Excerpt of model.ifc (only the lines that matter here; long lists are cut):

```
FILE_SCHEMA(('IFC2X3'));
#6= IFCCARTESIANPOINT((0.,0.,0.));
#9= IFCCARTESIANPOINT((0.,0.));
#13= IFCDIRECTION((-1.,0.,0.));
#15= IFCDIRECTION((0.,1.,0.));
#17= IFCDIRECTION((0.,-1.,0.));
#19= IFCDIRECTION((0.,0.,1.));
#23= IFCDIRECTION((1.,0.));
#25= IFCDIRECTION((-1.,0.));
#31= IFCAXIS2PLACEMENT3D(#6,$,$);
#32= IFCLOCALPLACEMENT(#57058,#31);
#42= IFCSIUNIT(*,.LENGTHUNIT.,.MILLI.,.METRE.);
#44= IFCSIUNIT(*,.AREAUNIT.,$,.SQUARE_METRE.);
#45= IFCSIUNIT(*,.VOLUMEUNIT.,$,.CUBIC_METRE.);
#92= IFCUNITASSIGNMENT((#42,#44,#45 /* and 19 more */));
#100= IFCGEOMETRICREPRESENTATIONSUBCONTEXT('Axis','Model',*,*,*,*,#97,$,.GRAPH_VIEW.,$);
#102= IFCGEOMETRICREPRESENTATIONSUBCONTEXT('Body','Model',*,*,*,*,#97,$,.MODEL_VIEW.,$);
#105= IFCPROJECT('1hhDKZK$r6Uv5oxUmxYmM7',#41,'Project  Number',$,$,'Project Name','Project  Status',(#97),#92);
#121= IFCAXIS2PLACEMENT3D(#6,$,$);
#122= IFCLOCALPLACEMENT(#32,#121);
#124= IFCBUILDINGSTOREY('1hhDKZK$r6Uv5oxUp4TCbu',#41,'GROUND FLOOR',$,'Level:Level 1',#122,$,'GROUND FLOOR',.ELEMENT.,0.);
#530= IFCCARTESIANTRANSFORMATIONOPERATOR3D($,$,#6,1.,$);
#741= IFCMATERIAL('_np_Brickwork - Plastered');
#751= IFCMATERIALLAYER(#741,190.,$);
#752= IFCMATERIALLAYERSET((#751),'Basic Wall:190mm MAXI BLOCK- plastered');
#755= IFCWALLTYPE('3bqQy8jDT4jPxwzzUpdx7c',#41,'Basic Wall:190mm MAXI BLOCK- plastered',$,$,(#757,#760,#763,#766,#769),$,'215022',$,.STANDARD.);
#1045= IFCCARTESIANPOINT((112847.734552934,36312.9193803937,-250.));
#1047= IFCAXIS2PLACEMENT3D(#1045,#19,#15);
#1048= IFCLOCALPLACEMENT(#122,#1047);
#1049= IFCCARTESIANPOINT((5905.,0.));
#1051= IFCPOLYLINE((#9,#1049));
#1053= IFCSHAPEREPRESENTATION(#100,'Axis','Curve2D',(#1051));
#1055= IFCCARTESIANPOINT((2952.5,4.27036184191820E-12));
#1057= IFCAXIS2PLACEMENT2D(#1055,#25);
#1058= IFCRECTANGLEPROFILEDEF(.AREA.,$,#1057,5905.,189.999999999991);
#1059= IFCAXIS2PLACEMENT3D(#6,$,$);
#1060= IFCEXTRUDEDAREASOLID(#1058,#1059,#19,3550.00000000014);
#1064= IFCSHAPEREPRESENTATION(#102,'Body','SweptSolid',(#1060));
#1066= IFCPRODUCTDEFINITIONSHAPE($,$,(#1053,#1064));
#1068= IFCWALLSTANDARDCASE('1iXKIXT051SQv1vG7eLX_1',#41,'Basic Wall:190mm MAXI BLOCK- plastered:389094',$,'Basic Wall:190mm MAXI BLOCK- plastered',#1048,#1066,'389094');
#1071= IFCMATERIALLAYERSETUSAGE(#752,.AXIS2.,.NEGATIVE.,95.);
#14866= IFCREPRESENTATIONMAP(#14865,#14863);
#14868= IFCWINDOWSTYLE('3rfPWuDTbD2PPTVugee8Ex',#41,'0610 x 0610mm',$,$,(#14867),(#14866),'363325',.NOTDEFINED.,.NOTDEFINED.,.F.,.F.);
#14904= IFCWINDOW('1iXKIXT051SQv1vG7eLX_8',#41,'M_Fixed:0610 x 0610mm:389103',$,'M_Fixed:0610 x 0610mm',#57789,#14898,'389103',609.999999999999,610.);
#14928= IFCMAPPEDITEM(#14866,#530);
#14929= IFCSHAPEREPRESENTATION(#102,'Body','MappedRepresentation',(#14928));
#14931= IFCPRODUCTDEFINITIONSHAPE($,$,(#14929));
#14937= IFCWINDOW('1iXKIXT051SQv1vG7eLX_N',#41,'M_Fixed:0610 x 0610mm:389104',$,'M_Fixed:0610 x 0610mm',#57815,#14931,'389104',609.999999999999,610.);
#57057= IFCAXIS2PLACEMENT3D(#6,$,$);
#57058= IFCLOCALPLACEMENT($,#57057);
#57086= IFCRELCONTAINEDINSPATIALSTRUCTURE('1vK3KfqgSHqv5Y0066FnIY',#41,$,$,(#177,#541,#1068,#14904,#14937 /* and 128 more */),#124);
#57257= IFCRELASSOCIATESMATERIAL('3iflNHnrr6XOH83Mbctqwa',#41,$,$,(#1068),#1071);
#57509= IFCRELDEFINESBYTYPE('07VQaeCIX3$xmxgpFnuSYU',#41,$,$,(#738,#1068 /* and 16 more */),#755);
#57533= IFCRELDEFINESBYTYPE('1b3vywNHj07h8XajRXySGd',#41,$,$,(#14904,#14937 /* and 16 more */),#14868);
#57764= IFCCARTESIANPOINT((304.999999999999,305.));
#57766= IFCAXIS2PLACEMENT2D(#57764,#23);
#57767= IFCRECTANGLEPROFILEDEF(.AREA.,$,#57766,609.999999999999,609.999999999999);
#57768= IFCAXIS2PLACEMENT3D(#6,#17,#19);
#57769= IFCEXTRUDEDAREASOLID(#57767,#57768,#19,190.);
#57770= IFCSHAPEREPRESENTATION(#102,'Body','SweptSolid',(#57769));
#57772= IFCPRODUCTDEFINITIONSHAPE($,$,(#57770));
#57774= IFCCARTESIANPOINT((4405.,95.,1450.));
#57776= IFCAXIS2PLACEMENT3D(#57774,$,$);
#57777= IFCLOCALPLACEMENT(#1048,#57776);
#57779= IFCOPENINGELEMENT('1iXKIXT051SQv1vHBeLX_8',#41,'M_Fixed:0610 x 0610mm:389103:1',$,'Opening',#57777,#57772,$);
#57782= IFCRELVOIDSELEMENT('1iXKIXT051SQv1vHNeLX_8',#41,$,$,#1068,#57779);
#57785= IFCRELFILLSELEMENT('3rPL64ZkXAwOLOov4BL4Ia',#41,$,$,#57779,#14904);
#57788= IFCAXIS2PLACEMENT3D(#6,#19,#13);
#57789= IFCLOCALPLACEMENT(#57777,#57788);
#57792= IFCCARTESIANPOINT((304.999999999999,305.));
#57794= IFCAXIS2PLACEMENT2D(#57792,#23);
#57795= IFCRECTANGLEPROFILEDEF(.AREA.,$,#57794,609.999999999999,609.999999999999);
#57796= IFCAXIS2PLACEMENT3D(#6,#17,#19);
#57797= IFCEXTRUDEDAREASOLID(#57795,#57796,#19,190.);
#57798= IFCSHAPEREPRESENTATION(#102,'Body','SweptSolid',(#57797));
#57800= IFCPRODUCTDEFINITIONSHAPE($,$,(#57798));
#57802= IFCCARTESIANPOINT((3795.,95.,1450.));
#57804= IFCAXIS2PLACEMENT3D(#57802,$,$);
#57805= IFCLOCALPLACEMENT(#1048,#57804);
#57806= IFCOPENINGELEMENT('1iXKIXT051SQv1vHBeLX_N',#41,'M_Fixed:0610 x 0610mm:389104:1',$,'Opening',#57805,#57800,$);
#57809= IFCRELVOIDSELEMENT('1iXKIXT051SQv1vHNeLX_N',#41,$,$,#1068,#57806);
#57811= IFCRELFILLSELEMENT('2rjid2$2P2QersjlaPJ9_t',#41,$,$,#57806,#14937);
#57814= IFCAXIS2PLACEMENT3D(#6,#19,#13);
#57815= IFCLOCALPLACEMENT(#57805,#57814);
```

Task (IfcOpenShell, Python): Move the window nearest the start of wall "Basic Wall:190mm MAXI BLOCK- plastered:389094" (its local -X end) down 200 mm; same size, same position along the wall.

```python
import numpy as np
import ifcopenshell
import ifcopenshell.api.geometry
import ifcopenshell.util.placement
import ifcopenshell.util.unit

model = ifcopenshell.open("model.ifc")
unit_scale = ifcopenshell.util.unit.calculate_unit_scale(model)

window = model.by_id(14937)
opening = window.FillsVoids[0].RelatingOpeningElement
dz = -0.2 / unit_scale

shift = np.array([0.0, 0.0, dz])
# The window is placed relative to its opening, so it follows when the opening moves.
matrix = ifcopenshell.util.placement.get_local_placement(opening.ObjectPlacement)
matrix[:3, 3] += shift
ifcopenshell.api.geometry.edit_object_placement(
    model, product=opening, matrix=matrix, is_si=False, should_transform_children=True
)

print(f"moved by {dz * unit_scale:+.3f} m")

model.write("model_edited.ifc")
```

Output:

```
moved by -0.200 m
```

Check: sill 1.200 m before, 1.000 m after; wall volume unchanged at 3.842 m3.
